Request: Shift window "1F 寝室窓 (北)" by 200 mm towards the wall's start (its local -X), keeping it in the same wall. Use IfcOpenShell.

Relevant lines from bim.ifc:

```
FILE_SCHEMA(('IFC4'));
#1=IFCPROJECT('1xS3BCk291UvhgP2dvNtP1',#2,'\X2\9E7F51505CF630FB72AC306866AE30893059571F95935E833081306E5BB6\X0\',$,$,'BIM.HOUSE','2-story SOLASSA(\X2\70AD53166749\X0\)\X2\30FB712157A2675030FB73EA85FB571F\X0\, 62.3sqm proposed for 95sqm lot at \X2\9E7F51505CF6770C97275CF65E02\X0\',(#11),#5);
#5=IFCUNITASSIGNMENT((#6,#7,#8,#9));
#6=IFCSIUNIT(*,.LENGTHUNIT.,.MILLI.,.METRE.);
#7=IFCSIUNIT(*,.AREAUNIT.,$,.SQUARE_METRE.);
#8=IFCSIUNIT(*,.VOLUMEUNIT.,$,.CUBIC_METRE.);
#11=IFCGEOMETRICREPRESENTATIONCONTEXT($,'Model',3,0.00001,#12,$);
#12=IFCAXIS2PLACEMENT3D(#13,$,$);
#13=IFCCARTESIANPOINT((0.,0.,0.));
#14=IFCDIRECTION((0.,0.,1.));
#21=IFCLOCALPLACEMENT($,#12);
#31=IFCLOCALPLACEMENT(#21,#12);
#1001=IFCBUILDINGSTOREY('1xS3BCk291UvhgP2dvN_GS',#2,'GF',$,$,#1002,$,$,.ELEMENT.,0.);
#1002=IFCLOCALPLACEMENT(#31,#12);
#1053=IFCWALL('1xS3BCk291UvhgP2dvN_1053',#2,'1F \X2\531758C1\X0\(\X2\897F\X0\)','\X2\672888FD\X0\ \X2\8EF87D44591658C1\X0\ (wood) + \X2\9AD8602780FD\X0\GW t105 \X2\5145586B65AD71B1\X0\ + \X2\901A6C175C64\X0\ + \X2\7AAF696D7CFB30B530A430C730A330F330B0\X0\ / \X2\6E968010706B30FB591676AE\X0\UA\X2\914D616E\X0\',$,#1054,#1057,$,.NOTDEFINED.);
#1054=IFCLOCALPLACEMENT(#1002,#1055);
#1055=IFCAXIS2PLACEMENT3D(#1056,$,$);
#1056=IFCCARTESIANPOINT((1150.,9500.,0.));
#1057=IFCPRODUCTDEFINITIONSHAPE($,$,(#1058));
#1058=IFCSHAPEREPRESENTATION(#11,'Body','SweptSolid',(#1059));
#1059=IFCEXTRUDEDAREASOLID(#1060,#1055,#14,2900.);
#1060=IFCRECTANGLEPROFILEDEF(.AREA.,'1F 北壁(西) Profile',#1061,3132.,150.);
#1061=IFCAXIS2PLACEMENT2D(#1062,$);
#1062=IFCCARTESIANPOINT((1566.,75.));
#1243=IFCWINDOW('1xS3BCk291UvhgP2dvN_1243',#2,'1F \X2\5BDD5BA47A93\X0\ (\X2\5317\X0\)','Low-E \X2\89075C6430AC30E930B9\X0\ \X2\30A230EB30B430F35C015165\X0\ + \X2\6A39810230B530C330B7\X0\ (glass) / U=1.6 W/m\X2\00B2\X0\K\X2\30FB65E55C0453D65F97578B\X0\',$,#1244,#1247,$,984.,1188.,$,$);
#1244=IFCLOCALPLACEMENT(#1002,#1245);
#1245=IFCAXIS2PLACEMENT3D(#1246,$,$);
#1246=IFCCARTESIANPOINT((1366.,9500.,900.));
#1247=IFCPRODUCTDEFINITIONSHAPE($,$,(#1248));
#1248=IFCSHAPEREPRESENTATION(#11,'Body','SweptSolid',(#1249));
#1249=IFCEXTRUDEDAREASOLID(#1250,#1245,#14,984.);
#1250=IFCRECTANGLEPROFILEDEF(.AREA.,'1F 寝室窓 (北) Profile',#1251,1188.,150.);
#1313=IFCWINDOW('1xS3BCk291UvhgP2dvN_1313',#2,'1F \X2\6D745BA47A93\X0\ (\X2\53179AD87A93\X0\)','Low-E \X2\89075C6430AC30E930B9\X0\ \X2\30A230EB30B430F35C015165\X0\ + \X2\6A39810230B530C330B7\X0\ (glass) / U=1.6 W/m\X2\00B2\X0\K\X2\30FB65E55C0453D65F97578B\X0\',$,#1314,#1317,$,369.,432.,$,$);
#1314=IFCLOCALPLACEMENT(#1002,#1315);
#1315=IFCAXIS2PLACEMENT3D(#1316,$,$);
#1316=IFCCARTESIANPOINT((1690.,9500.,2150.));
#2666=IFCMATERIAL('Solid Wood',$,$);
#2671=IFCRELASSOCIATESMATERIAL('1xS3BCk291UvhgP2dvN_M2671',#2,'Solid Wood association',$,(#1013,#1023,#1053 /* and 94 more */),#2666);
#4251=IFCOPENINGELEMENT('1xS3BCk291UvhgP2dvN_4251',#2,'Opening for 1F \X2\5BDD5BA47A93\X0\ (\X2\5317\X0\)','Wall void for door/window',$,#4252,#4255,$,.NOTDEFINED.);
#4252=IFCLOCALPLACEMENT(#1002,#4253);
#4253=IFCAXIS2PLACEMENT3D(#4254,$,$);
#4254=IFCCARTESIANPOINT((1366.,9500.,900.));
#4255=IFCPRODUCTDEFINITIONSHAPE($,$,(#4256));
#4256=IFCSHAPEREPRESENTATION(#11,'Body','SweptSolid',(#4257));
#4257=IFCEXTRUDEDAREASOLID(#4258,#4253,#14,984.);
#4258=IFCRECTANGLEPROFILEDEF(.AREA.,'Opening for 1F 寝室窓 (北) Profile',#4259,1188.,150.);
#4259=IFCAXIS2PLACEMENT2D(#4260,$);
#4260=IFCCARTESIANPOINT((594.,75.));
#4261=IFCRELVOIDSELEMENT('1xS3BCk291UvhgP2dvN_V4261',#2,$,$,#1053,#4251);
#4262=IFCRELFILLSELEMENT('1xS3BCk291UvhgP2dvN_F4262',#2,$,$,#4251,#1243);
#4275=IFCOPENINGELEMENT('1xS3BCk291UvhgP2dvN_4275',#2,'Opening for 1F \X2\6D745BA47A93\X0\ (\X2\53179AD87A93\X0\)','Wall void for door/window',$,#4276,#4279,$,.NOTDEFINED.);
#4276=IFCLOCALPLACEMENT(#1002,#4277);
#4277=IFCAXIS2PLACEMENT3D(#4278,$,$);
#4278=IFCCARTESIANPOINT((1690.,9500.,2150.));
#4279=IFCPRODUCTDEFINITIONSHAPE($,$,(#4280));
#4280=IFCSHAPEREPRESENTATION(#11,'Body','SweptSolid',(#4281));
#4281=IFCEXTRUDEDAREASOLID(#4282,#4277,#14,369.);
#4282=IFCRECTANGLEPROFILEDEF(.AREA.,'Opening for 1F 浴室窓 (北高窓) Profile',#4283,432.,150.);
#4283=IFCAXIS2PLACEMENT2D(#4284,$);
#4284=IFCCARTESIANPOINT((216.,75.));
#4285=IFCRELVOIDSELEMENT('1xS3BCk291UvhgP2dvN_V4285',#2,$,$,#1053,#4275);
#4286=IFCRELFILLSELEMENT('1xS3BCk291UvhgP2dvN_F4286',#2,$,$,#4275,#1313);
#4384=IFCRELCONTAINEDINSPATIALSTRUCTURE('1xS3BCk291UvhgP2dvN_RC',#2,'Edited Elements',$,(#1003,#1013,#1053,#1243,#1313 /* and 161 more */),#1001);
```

```python
import ifcopenshell
import ifcopenshell.api.geometry
import ifcopenshell.util.placement
import ifcopenshell.util.unit

model = ifcopenshell.open("bim.ifc")
unit_scale = ifcopenshell.util.unit.calculate_unit_scale(model)

window = model.by_id(1243)
opening = window.FillsVoids[0].RelatingOpeningElement
wall = opening.VoidsElements[0].RelatingBuildingElement

wall_matrix = ifcopenshell.util.placement.get_local_placement(wall.ObjectPlacement)
shift = wall_matrix[:3, 0] * -0.2 / unit_scale
before = ifcopenshell.util.placement.get_local_placement(window.ObjectPlacement)[:3, 3].copy()

# The window is not placed relative to its opening, so move both.
for product in (opening, window):
    matrix = ifcopenshell.util.placement.get_local_placement(product.ObjectPlacement)
    matrix[:3, 3] += shift
    ifcopenshell.api.geometry.edit_object_placement(model, product=product, matrix=matrix, is_si=False)

after = ifcopenshell.util.placement.get_local_placement(window.ObjectPlacement)[:3, 3]
print("window moved by", (after - before).round(3) + 0.0)

model.write("bim-out.ifc")
```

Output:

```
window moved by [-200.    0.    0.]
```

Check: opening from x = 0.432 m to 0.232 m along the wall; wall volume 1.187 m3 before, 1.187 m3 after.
